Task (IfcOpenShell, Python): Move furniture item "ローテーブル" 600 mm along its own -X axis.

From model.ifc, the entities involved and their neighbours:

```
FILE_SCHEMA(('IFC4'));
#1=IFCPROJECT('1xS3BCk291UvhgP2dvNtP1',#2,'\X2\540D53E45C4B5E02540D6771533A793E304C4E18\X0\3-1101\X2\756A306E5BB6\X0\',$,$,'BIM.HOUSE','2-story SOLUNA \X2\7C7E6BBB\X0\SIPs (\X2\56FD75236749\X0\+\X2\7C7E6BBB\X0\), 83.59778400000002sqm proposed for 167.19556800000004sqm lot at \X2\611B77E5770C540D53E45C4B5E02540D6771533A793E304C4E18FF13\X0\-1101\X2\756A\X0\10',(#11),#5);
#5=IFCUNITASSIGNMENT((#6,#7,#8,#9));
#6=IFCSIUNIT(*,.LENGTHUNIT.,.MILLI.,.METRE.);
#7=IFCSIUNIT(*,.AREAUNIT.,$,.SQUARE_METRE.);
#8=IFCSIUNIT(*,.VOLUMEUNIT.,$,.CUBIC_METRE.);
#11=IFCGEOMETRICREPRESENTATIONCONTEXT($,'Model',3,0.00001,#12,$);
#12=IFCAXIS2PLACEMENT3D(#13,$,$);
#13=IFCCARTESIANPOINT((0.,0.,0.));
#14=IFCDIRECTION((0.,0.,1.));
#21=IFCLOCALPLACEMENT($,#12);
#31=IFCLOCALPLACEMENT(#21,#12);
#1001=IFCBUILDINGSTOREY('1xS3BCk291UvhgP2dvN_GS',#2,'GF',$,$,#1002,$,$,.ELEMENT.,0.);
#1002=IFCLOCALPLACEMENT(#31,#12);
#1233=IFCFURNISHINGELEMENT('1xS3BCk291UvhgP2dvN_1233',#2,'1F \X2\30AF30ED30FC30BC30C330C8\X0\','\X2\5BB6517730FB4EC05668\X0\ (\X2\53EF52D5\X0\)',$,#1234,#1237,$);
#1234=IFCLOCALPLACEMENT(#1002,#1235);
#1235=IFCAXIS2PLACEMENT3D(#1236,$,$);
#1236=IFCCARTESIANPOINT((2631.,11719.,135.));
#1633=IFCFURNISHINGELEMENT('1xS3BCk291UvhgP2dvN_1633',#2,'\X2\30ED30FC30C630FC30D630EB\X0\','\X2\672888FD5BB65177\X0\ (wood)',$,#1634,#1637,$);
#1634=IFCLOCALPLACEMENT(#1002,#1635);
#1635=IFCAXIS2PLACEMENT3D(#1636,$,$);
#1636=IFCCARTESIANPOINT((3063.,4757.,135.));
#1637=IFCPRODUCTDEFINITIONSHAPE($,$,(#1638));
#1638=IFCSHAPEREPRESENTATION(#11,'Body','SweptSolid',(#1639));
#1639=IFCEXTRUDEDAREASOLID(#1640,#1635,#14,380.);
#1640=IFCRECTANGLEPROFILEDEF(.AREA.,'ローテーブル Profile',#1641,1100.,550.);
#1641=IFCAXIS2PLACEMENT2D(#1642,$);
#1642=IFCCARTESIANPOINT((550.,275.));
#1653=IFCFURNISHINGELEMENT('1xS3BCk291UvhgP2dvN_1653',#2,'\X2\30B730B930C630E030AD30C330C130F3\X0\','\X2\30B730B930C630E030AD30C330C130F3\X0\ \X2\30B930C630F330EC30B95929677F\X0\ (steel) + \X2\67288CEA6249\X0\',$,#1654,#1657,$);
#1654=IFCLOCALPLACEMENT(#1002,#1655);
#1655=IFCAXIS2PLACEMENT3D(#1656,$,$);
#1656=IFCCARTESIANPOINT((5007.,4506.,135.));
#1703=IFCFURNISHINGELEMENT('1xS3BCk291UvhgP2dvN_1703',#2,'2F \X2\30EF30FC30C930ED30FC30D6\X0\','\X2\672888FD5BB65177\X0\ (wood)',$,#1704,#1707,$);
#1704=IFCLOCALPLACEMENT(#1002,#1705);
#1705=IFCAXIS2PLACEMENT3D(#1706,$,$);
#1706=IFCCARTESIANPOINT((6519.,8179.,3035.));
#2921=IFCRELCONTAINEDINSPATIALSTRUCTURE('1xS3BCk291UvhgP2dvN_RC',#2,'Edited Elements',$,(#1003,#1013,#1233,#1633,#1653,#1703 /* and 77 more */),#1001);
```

```python
import ifcopenshell
import ifcopenshell.api.geometry
import ifcopenshell.util.placement

model = ifcopenshell.open("model.ifc")

item = model.by_id(1633)
matrix = ifcopenshell.util.placement.get_local_placement(item.ObjectPlacement)
matrix[:3, 3] -= matrix[:3, 0] * 600.0
ifcopenshell.api.geometry.edit_object_placement(model, product=item, matrix=matrix, is_si=False)

print(ifcopenshell.util.placement.get_local_placement(item.ObjectPlacement).round(3) + 0.0)

model.write("model-out.ifc")
```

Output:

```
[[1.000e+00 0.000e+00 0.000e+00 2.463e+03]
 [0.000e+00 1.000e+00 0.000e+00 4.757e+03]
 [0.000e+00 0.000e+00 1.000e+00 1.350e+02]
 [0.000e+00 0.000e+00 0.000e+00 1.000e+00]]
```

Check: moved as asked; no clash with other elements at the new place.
